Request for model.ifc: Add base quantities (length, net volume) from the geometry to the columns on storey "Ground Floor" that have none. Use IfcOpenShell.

First a look at what the model holds.

```python
import ifcopenshell
import ifcopenshell.util.element
import ifcopenshell.util.unit

model = ifcopenshell.open("model.ifc")
print(model.schema)
for unit_type in ("LENGTHUNIT", "AREAUNIT", "VOLUMEUNIT"):
    print(unit_type, ifcopenshell.util.unit.calculate_unit_scale(model, unit_type))
storey = next(s for s in model.by_type("IfcBuildingStorey") if s.Name == "Ground Floor")
columns = [e for e in ifcopenshell.util.element.get_decomposition(storey) if e.is_a("IfcColumn")]
for e in sorted(columns, key=lambda e: e.id()):
    print(e.id(), e.is_a(), e.Name, list(ifcopenshell.util.element.get_psets(e, qtos_only=True)), sep=" | ")
```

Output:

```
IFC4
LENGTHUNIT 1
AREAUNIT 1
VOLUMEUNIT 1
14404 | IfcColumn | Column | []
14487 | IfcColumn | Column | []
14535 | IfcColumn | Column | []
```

```python
import ifcopenshell
import ifcopenshell.api.pset
import ifcopenshell.geom
import ifcopenshell.util.element
import ifcopenshell.util.shape
import ifcopenshell.util.unit

model = ifcopenshell.open("model.ifc")
unit_scale = ifcopenshell.util.unit.calculate_unit_scale(model)
volume_scale = ifcopenshell.util.unit.calculate_unit_scale(model, "VOLUMEUNIT")
settings = ifcopenshell.geom.settings()

storey = next(s for s in model.by_type("IfcBuildingStorey") if s.Name == "Ground Floor")
columns = [e for e in ifcopenshell.util.element.get_decomposition(storey) if e.is_a("IfcColumn")]

for e in sorted(columns, key=lambda e: e.id()):
    if ifcopenshell.util.element.get_psets(e, qtos_only=True, should_inherit=False):
        continue
    # Geometry comes back in metres, in the element's own axes.
    shape = ifcopenshell.geom.create_shape(settings, e)
    values = {
        "Length": ifcopenshell.util.shape.get_z(shape.geometry) / unit_scale,
        "NetVolume": ifcopenshell.util.shape.get_volume(shape.geometry) / volume_scale,
    }
    qto = ifcopenshell.api.pset.add_qto(model, product=e, name="Qto_ColumnBaseQuantities")
    ifcopenshell.api.pset.edit_qto(model, qto=qto, properties=values)
    print(e.id(), {k: round(v, 3) for k, v in values.items()})

model.write("model_v2.ifc")
```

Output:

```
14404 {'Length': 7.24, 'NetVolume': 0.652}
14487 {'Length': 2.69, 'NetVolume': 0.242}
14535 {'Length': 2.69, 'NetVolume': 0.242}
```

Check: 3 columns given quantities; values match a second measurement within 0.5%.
